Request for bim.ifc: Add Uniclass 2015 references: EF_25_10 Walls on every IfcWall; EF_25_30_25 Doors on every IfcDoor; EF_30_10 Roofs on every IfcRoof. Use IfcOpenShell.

First a look at what the model holds.

```python
import ifcopenshell

model = ifcopenshell.open("bim.ifc")
print(model.schema)
print("classifications:", [c.Name for c in model.by_type("IfcClassification")])
for ifc_class in ("IfcDoor", "IfcRoof", "IfcStair", "IfcWall", "IfcWindow"):
    print(ifc_class, len(model.by_type(ifc_class)))
```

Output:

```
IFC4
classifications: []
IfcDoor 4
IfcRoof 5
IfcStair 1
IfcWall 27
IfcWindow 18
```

```python
import ifcopenshell
import ifcopenshell.api.classification

model = ifcopenshell.open("bim.ifc")

system = ifcopenshell.api.classification.add_classification(model, classification="Uniclass 2015")

codes = {
    "IfcWall": ("EF_25_10", "Walls"),
    "IfcDoor": ("EF_25_30_25", "Doors"),
    "IfcRoof": ("EF_30_10", "Roofs"),
}
for ifc_class, (code, name) in codes.items():
    products = model.by_type(ifc_class)
    ifcopenshell.api.classification.add_reference(
        model, products=products, classification=system, identification=code, name=name
    )
    print(code, len(products))

model.write("bim-out.ifc")
```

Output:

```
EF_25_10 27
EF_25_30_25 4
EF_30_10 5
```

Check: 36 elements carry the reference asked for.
